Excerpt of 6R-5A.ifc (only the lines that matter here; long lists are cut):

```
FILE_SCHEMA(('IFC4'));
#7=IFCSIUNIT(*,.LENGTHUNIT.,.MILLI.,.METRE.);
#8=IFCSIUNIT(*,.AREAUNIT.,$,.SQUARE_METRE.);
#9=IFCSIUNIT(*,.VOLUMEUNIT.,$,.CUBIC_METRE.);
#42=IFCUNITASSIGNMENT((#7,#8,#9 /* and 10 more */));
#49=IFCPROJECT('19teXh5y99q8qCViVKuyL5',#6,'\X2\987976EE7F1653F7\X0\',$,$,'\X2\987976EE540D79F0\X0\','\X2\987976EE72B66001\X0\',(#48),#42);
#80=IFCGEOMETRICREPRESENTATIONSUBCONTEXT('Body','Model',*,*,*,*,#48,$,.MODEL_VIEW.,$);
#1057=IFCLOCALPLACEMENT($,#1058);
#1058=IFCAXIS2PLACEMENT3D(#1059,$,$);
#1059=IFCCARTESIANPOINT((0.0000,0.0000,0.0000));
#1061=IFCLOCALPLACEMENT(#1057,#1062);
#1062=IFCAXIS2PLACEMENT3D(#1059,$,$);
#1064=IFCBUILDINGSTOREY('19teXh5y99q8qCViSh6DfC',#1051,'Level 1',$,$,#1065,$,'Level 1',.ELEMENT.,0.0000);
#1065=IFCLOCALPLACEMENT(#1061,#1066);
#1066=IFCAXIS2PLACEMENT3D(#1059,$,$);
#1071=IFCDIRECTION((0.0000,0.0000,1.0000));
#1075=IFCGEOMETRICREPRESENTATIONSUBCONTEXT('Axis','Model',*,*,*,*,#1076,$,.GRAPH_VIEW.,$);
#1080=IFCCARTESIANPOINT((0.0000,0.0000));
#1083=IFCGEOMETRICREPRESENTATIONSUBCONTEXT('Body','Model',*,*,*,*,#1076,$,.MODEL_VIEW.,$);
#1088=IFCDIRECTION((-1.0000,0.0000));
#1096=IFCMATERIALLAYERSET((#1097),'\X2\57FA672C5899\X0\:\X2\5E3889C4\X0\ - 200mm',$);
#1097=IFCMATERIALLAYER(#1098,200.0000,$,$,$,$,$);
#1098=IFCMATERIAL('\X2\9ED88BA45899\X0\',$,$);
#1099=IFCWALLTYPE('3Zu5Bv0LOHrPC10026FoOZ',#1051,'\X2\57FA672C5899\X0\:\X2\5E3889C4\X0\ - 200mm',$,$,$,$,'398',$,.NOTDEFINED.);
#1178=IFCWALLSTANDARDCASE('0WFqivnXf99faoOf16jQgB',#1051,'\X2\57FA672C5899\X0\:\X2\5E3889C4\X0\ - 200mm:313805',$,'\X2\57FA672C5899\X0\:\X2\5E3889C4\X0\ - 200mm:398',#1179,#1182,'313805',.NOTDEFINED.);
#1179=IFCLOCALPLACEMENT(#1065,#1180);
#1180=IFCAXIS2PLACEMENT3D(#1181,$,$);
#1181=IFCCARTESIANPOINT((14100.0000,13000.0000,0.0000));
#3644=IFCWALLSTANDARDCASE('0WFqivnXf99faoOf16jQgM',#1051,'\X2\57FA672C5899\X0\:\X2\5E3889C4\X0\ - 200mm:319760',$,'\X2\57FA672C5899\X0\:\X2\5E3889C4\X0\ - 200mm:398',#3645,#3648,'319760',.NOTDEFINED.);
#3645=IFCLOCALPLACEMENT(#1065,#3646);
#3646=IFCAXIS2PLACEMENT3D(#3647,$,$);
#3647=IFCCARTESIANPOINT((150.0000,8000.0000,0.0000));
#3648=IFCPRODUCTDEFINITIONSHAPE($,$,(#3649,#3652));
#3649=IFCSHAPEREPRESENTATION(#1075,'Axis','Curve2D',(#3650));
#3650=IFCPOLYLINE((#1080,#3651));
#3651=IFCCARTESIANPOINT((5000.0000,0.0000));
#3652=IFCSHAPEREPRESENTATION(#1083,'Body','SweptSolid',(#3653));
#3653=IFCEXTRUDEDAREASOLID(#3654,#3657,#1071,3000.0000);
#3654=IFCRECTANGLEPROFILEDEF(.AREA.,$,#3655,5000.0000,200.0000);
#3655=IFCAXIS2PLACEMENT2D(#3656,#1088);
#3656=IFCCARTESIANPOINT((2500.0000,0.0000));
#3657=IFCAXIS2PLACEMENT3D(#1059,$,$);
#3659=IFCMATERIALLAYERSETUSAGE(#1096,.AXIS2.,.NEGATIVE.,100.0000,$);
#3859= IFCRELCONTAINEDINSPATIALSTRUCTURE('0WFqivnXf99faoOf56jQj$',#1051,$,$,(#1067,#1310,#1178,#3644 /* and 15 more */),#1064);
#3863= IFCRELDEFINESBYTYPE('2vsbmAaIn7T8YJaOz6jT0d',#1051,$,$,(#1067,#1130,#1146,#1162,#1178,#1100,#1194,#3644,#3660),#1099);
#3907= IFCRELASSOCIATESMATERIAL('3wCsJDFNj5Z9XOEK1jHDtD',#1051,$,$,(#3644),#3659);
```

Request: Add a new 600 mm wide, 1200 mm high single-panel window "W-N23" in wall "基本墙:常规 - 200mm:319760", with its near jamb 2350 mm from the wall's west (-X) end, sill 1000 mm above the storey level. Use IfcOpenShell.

```python
import numpy as np
import ifcopenshell
import ifcopenshell.api.feature
import ifcopenshell.api.geometry
import ifcopenshell.api.root
import ifcopenshell.api.spatial
import ifcopenshell.geom
import ifcopenshell.util.element
import ifcopenshell.util.placement
import ifcopenshell.util.representation
import ifcopenshell.util.shape
import ifcopenshell.util.unit

model = ifcopenshell.open("6R-5A.ifc")
unit_scale = ifcopenshell.util.unit.calculate_unit_scale(model)
settings = ifcopenshell.geom.settings()


def volume(element):
    """Net volume in cubic metres, openings subtracted."""
    shape = ifcopenshell.geom.create_shape(settings, element)
    return ifcopenshell.util.shape.get_volume(shape.geometry)


wall = model.by_guid("0WFqivnXf99faoOf16jQgM")
storey = ifcopenshell.util.element.get_container(wall, ifc_class="IfcBuildingStorey")
context = ifcopenshell.util.representation.get_context(model, "Model", "Body", "MODEL_VIEW")
before = volume(wall)

width, height, from_end, sill = 0.6, 1.2, 2.35, 1  # metres

# The wall runs along its own X axis, and the end named is its -X end.
wall_shape = ifcopenshell.geom.create_shape(settings, wall)
x, y, z = ifcopenshell.util.shape.get_vertices(wall_shape.geometry).T
start = x.min() + from_end
face, thickness = float(y.min()), float(y.max() - y.min())
wall_matrix = ifcopenshell.util.placement.get_local_placement(wall.ObjectPlacement)
level = ifcopenshell.util.placement.get_local_placement(storey.ObjectPlacement)[2, 3]


def in_wall(x, y):
    """Placement at x, y metres in the wall's axes, at sill height."""
    matrix = wall_matrix.copy()
    matrix[:, 3] = wall_matrix @ np.array([x / unit_scale, y / unit_scale, 0.0, 1.0])
    matrix[2, 3] = level + sill / unit_scale
    return matrix


# Opening: a box that overshoots both wall faces by 50 mm.
opening = ifcopenshell.api.root.create_entity(model, ifc_class="IfcOpeningElement", predefined_type="OPENING")
box = ifcopenshell.api.geometry.add_wall_representation(
    model, context=context, length=width, height=height, thickness=thickness + 0.1
)
ifcopenshell.api.geometry.assign_representation(model, product=opening, representation=box)
ifcopenshell.api.geometry.edit_object_placement(model, product=opening, matrix=in_wall(start, face - 0.05), is_si=False)
ifcopenshell.api.feature.add_feature(model, feature=opening, element=wall)

window = ifcopenshell.api.root.create_entity(model, ifc_class="IfcWindow", name="W-N23", predefined_type="WINDOW")
window.OverallWidth, window.OverallHeight = width / unit_scale, height / unit_scale
window.PartitioningType = "SINGLE_PANEL"
body = ifcopenshell.api.geometry.add_window_representation(
    model,
    context=context,
    overall_width=window.OverallWidth,
    overall_height=window.OverallHeight,
    partition_type="SINGLE_PANEL",
)
ifcopenshell.api.geometry.assign_representation(model, product=window, representation=body)
ifcopenshell.api.spatial.assign_container(model, products=[window], relating_structure=storey)
ifcopenshell.api.feature.add_filling(model, opening=opening, element=window)

# Centre the window in the wall's thickness.
ifcopenshell.api.geometry.edit_object_placement(model, product=window, matrix=in_wall(start, face), is_si=False)
window_shape = ifcopenshell.geom.create_shape(settings, window)
depth = ifcopenshell.util.shape.get_vertices(window_shape.geometry)[:, 1]
offset = face + thickness / 2 - (depth.min() + depth.max()) / 2
ifcopenshell.api.geometry.edit_object_placement(model, product=window, matrix=in_wall(start, offset), is_si=False)

after = volume(wall)

print(f"wall volume {before:.3f} -> {after:.3f} m3")

model.write("6R-5A-out.ifc")
```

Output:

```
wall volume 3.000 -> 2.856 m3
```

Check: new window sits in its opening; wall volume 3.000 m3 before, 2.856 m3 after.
